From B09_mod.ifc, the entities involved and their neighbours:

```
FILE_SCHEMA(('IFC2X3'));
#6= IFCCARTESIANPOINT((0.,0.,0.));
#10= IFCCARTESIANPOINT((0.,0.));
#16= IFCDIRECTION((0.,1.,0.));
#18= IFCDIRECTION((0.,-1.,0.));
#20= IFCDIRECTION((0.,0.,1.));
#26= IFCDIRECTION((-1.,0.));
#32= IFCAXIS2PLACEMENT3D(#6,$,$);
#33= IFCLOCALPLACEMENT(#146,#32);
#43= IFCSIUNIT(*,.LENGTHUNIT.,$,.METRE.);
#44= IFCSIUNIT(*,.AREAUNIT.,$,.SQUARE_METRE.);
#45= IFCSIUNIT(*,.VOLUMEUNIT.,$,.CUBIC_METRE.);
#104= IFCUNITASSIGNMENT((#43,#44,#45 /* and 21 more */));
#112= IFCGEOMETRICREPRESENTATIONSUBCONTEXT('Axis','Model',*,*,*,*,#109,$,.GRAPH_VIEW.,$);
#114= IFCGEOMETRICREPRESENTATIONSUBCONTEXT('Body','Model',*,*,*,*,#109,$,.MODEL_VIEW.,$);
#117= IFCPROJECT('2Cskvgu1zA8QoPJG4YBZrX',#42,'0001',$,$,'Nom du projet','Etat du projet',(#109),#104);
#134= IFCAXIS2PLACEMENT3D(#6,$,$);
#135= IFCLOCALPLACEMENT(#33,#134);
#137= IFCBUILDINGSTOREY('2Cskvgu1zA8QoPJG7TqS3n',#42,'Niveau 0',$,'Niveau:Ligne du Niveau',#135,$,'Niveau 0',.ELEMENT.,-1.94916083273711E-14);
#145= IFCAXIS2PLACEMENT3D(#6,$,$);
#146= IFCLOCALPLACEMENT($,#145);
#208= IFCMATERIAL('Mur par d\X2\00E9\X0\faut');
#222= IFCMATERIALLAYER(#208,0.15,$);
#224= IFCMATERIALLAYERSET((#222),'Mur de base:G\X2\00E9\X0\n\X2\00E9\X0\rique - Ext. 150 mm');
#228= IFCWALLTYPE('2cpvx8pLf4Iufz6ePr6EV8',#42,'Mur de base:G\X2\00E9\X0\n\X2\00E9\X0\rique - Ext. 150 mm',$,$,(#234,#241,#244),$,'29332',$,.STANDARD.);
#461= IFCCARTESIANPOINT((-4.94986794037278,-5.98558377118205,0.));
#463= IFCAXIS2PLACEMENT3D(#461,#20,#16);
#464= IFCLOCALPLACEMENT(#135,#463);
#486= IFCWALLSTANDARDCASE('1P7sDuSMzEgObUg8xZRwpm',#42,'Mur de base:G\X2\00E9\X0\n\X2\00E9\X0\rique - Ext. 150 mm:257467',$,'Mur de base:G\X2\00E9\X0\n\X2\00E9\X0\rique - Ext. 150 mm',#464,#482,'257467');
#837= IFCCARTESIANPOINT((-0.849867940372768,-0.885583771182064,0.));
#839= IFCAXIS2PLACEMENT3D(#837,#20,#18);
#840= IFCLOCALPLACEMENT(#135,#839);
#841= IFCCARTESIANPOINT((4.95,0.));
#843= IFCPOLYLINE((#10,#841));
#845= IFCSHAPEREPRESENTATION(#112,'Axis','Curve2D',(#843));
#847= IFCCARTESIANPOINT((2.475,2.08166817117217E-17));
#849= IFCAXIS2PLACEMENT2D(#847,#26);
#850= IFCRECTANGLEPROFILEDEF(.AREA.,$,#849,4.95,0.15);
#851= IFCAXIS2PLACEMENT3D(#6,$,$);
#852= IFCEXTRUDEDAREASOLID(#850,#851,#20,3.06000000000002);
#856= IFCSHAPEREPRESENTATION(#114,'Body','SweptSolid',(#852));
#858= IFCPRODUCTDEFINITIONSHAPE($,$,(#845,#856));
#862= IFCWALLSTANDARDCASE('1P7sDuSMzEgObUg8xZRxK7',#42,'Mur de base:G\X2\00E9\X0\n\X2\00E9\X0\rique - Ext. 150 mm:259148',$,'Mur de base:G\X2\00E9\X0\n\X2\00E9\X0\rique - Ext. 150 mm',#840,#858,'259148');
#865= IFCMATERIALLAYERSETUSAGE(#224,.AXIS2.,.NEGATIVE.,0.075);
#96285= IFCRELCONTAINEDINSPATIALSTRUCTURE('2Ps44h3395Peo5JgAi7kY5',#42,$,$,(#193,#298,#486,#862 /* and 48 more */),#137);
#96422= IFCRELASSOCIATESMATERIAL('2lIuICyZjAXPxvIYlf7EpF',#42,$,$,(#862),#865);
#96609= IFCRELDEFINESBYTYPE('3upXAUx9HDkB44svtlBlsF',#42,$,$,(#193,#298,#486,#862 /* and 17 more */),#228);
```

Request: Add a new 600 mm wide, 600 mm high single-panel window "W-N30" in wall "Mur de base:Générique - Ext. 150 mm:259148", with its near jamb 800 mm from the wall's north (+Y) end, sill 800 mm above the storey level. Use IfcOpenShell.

```python
import numpy as np
import ifcopenshell
import ifcopenshell.api.feature
import ifcopenshell.api.geometry
import ifcopenshell.api.root
import ifcopenshell.api.spatial
import ifcopenshell.api.type
import ifcopenshell.geom
import ifcopenshell.util.element
import ifcopenshell.util.placement
import ifcopenshell.util.representation
import ifcopenshell.util.shape
import ifcopenshell.util.unit

model = ifcopenshell.open("B09_mod.ifc")
unit_scale = ifcopenshell.util.unit.calculate_unit_scale(model)
settings = ifcopenshell.geom.settings()


def volume(element):
    """Net volume in cubic metres, openings subtracted."""
    shape = ifcopenshell.geom.create_shape(settings, element)
    return ifcopenshell.util.shape.get_volume(shape.geometry)


wall = model.by_id(862)
storey = ifcopenshell.util.element.get_container(wall, ifc_class="IfcBuildingStorey")
context = ifcopenshell.util.representation.get_context(model, "Model", "Body", "MODEL_VIEW")
before = volume(wall)

width, height, from_end, sill = 0.6, 0.6, 0.8, 0.8  # metres

# The wall runs along its own X axis, and the end named is its -X end.
wall_shape = ifcopenshell.geom.create_shape(settings, wall)
x, y, z = ifcopenshell.util.shape.get_vertices(wall_shape.geometry).T
start = x.min() + from_end
face, thickness = float(y.min()), float(y.max() - y.min())
wall_matrix = ifcopenshell.util.placement.get_local_placement(wall.ObjectPlacement)
level = ifcopenshell.util.placement.get_local_placement(storey.ObjectPlacement)[2, 3]


def in_wall(x, y):
    """Placement at x, y metres in the wall's axes, at sill height."""
    matrix = wall_matrix.copy()
    matrix[:, 3] = wall_matrix @ np.array([x / unit_scale, y / unit_scale, 0.0, 1.0])
    matrix[2, 3] = level + sill / unit_scale
    return matrix


# Opening: a box that overshoots both wall faces by 50 mm.
opening = ifcopenshell.api.root.create_entity(model, ifc_class="IfcOpeningElement")
box = ifcopenshell.api.geometry.add_wall_representation(
    model, context=context, length=width, height=height, thickness=thickness + 0.1
)
ifcopenshell.api.geometry.assign_representation(model, product=opening, representation=box)
ifcopenshell.api.geometry.edit_object_placement(model, product=opening, matrix=in_wall(start, face - 0.05), is_si=False)
ifcopenshell.api.feature.add_feature(model, feature=opening, element=wall)

window = ifcopenshell.api.root.create_entity(model, ifc_class="IfcWindow", name="W-N30")
window.OverallWidth, window.OverallHeight = width / unit_scale, height / unit_scale
body = ifcopenshell.api.geometry.add_window_representation(
    model,
    context=context,
    overall_width=window.OverallWidth,
    overall_height=window.OverallHeight,
    partition_type="SINGLE_PANEL",
)
ifcopenshell.api.geometry.assign_representation(model, product=window, representation=body)
ifcopenshell.api.spatial.assign_container(model, products=[window], relating_structure=storey)
fills = ifcopenshell.api.feature.add_filling(model, opening=opening, element=window)
fills.OwnerHistory = window.OwnerHistory  # required in IFC2X3

# IFC2X3 keeps the operation on the window style.
style = ifcopenshell.api.root.create_entity(model, ifc_class="IfcWindowStyle", name="W-N30")
style.OperationType, style.ConstructionType = "SINGLE_PANEL", "NOTDEFINED"
style.ParameterTakesPrecedence = style.Sizeable = False
ifcopenshell.api.type.assign_type(model, related_objects=[window], relating_type=style)

# Centre the window in the wall's thickness.
ifcopenshell.api.geometry.edit_object_placement(model, product=window, matrix=in_wall(start, face), is_si=False)
window_shape = ifcopenshell.geom.create_shape(settings, window)
depth = ifcopenshell.util.shape.get_vertices(window_shape.geometry)[:, 1]
offset = face + thickness / 2 - (depth.min() + depth.max()) / 2
ifcopenshell.api.geometry.edit_object_placement(model, product=window, matrix=in_wall(start, offset), is_si=False)

after = volume(wall)

print(f"wall volume {before:.3f} -> {after:.3f} m3")

model.write("B09_mod_updated.ifc")
```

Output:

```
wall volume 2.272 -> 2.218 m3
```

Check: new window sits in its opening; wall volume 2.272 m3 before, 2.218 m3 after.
